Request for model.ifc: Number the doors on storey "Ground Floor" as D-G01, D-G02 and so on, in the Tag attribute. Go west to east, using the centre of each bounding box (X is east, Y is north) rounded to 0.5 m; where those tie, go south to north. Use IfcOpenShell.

First a look at what the model holds.

```python
import ifcopenshell
import ifcopenshell.util.element
import ifcopenshell.util.placement

model = ifcopenshell.open("model.ifc")
print(model.schema)
storey = next(s for s in model.by_type("IfcBuildingStorey") if s.Name == "Ground Floor")
doors = [e for e in ifcopenshell.util.element.get_decomposition(storey) if e.is_a("IfcDoor")]
for e in sorted(doors, key=lambda e: e.id()):
    origin = ifcopenshell.util.placement.get_local_placement(e.ObjectPlacement)[:3, 3]
    print(e.id(), e.Tag, e.Name, origin.round(2) + 0.0, sep=" | ")
```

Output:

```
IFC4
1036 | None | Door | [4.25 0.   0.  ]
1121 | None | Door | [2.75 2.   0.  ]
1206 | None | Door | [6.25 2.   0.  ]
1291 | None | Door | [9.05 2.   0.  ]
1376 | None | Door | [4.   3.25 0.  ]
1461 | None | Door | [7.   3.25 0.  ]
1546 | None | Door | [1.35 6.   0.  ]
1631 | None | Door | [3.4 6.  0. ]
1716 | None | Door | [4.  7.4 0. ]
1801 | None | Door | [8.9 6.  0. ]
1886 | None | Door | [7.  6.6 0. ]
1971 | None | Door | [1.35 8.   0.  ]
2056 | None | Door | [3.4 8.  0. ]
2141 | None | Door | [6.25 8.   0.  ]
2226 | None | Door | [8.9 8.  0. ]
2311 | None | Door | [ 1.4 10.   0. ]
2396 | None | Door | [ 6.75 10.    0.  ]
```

```python
import ifcopenshell
import ifcopenshell.geom
import ifcopenshell.util.element
import ifcopenshell.util.shape

model = ifcopenshell.open("model.ifc")
settings = ifcopenshell.geom.settings()
settings.set("use-world-coords", True)


def centre(element):
    shape = ifcopenshell.geom.create_shape(settings, element)
    return ifcopenshell.util.shape.get_bbox_centroid(shape.geometry)


storey = next(s for s in model.by_type("IfcBuildingStorey") if s.Name == "Ground Floor")
doors = [e for e in ifcopenshell.util.element.get_decomposition(storey) if e.is_a("IfcDoor")]

# Insertion points can sit at a corner or the storey origin, so sort by the geometry (in metres).
centres = {e: centre(e) for e in doors}
doors.sort(key=lambda e: (round(centres[e][0] / 0.5), centres[e][1]))

for i, e in enumerate(doors, start=1):
    number = f"D-G{i:02d}"
    e.Tag = number
    print(e.id(), number)

model.write("model_updated.ifc")
```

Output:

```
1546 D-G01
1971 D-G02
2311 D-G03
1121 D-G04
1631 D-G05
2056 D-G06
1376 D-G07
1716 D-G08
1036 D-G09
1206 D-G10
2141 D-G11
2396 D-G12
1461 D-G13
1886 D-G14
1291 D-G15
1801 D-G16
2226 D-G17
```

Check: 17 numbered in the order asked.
